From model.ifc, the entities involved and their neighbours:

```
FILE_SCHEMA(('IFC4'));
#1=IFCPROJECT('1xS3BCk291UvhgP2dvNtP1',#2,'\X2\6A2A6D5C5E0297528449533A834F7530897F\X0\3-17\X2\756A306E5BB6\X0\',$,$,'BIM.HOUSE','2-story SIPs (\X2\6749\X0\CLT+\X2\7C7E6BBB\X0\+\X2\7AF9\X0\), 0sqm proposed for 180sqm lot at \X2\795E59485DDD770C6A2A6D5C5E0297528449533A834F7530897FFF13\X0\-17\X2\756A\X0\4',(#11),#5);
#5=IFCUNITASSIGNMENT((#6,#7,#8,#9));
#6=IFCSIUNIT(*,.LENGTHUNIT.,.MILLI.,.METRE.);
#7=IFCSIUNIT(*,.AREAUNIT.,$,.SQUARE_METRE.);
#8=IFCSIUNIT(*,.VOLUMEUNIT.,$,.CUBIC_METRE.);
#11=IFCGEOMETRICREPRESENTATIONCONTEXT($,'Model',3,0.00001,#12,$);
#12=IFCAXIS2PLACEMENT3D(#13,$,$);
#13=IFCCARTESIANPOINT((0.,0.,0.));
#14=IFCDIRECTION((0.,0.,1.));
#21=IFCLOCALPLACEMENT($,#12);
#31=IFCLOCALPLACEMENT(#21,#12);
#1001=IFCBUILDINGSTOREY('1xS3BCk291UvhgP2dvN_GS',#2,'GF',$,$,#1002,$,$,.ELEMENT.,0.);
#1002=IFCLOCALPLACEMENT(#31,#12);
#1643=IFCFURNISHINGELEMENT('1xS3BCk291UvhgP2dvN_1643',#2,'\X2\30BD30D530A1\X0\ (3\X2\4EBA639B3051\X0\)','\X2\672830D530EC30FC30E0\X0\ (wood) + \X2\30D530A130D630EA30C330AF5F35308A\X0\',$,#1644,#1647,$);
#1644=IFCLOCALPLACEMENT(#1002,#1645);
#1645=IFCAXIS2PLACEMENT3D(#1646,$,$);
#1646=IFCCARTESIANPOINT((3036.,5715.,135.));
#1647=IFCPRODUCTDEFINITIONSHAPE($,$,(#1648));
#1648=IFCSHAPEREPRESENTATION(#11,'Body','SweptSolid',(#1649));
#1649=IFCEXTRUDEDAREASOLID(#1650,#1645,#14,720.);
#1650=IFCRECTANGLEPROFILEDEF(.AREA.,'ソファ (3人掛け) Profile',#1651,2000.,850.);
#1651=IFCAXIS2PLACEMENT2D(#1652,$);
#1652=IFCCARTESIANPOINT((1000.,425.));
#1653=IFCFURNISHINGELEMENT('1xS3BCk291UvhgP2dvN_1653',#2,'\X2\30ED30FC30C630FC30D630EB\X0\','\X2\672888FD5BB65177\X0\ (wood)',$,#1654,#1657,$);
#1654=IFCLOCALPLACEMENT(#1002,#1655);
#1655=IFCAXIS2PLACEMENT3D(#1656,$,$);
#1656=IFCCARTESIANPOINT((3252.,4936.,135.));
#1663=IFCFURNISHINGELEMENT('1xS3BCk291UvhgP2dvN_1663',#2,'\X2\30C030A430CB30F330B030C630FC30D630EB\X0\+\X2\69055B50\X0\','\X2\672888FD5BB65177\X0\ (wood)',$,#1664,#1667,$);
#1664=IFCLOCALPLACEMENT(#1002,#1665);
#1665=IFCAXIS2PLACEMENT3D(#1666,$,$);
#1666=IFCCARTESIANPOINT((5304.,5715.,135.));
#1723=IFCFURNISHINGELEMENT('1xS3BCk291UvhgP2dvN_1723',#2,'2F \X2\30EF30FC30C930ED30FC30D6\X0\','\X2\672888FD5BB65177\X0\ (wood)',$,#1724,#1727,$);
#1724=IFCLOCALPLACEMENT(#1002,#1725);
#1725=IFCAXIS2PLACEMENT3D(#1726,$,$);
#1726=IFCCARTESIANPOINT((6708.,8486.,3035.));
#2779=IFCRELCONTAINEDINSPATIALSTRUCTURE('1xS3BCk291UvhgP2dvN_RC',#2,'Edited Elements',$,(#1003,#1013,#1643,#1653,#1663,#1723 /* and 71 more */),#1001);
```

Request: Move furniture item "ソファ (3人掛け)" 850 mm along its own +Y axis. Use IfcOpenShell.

```python
import ifcopenshell
import ifcopenshell.api.geometry
import ifcopenshell.util.placement

model = ifcopenshell.open("model.ifc")

item = model.by_guid("1xS3BCk291UvhgP2dvN_1643")
matrix = ifcopenshell.util.placement.get_local_placement(item.ObjectPlacement)
matrix[:3, 3] += matrix[:3, 1] * 850.0
ifcopenshell.api.geometry.edit_object_placement(model, product=item, matrix=matrix, is_si=False)

print(ifcopenshell.util.placement.get_local_placement(item.ObjectPlacement).round(3) + 0.0)

model.write("model_updated.ifc")
```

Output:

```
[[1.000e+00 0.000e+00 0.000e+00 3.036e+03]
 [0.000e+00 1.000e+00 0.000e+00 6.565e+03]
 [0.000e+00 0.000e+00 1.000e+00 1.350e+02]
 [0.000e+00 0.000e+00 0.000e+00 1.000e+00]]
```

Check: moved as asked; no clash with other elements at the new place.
